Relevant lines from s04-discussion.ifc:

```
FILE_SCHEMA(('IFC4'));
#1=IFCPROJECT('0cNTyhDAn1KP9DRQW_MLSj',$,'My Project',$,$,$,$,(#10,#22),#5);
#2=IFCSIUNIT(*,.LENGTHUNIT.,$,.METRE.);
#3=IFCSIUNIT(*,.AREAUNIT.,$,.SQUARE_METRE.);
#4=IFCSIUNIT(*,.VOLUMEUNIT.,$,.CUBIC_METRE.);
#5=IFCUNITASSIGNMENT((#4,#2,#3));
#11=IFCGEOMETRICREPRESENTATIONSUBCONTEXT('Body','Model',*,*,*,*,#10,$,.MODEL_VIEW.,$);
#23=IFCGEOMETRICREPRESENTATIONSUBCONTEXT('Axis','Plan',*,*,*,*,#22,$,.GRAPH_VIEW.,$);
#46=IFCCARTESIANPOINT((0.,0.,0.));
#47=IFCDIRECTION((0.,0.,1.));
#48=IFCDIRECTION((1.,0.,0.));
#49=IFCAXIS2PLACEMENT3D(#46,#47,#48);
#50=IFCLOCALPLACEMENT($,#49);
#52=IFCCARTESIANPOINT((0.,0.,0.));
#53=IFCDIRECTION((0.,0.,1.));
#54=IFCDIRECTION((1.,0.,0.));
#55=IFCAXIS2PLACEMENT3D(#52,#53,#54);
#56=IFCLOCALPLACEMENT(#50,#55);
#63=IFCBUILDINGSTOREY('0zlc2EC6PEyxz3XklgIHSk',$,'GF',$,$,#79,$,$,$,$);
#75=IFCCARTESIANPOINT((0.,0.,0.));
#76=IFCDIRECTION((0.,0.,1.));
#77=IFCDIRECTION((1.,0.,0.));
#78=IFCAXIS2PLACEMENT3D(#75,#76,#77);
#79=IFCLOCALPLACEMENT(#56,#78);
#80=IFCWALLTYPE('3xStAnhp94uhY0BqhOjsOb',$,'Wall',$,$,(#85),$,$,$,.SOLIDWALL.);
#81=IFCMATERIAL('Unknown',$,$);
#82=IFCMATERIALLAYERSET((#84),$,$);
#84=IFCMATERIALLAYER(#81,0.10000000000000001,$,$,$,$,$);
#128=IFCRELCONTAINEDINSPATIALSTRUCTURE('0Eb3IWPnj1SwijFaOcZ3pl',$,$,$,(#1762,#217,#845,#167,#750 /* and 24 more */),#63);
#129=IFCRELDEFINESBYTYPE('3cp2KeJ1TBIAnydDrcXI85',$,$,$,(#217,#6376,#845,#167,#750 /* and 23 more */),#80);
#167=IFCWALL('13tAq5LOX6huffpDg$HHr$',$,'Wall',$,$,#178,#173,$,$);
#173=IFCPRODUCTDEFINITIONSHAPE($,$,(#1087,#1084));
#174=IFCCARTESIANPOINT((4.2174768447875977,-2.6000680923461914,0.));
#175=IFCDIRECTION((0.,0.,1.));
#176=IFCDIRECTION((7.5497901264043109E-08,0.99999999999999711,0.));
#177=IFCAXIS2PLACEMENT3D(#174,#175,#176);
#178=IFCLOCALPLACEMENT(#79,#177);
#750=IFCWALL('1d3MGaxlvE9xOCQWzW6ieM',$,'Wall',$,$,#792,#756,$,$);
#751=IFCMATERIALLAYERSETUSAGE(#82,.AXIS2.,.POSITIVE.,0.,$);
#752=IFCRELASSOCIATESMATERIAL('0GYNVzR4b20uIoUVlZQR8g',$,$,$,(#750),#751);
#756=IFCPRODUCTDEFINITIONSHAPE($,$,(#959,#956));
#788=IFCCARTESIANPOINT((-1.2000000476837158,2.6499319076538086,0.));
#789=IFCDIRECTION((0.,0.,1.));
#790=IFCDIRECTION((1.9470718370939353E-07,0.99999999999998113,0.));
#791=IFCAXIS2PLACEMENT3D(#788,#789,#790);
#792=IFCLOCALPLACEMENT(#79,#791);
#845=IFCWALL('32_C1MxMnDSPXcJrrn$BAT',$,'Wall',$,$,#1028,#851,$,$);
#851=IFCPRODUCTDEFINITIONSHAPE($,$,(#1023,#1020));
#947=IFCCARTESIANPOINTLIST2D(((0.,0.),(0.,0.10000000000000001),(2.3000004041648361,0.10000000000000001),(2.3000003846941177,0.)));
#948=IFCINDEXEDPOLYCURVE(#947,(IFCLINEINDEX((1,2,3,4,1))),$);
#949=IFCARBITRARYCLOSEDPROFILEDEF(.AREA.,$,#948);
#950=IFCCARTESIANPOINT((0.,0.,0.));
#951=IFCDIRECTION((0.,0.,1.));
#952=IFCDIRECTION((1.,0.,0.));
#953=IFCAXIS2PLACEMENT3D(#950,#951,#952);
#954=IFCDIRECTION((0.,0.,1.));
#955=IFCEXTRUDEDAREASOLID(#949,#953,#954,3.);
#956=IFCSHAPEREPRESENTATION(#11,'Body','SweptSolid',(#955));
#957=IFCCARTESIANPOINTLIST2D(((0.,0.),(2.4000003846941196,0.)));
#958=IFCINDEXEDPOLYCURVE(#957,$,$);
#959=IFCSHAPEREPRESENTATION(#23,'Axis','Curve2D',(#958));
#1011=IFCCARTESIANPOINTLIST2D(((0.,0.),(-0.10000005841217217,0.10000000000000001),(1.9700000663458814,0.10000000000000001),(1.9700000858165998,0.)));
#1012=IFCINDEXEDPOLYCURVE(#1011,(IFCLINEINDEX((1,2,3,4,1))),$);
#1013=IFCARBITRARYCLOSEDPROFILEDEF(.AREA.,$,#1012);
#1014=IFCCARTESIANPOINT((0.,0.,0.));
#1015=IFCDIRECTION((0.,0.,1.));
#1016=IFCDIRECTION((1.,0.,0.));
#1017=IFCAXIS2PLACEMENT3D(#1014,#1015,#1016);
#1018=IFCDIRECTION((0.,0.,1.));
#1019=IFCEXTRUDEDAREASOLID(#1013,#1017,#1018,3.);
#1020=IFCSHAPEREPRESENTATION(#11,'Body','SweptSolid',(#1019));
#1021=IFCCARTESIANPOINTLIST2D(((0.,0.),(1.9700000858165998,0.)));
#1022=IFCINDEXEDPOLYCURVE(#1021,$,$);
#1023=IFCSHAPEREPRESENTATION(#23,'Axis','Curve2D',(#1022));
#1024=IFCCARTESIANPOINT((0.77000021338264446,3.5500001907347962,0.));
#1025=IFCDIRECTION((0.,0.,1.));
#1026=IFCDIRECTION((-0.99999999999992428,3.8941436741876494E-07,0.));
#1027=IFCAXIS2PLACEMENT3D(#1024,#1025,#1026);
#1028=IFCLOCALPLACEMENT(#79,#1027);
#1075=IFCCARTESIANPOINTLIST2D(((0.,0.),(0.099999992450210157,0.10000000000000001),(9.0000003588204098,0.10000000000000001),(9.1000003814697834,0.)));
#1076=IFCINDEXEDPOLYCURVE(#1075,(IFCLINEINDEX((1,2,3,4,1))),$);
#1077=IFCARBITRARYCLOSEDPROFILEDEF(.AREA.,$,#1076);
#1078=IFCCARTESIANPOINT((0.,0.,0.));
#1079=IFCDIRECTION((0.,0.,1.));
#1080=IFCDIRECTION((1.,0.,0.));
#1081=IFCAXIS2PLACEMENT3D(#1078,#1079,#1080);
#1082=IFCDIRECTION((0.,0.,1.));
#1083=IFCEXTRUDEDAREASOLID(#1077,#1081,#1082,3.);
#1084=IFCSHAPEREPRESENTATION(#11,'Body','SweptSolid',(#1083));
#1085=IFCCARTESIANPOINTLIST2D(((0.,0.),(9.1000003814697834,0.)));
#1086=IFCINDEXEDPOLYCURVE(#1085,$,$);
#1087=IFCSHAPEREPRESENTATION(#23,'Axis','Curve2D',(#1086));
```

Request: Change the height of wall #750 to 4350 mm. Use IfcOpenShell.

```python
import ifcopenshell
import ifcopenshell.geom
import ifcopenshell.util.representation
import ifcopenshell.util.shape

model = ifcopenshell.open("s04-discussion.ifc")
settings = ifcopenshell.geom.settings()


def volume(element):
    """Net volume in cubic metres, openings subtracted."""
    shape = ifcopenshell.geom.create_shape(settings, element)
    return ifcopenshell.util.shape.get_volume(shape.geometry)


wall = model.by_guid("1d3MGaxlvE9xOCQWzW6ieM")
before = volume(wall)

body = ifcopenshell.util.representation.get_representation(wall, "Model", "Body")
solid = body.Items[0]
old_height = solid.Depth
solid.Depth = 4.35
after = volume(wall)

print(f"height {old_height:g} -> {solid.Depth:g}, volume {before:.3f} -> {after:.3f} m3")

model.write("s04-discussion-out.ifc")
```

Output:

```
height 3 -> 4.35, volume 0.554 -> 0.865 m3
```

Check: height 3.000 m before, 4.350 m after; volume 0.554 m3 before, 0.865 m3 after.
